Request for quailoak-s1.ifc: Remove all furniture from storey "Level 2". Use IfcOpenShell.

First a look at what the model holds.

```python
import ifcopenshell
import ifcopenshell.util.element

model = ifcopenshell.open("quailoak-s1.ifc")
print(model.schema)
storey = next(s for s in model.by_type("IfcBuildingStorey") if s.Name == "Level 2")
furniture = [e for e in ifcopenshell.util.element.get_decomposition(storey) if e.is_a("IfcFurnishingElement")]
seen = {}
for e in furniture:
    element_type = ifcopenshell.util.element.get_type(e)
    name = element_type.Name if element_type not in (None, e) else None
    seen[name] = seen.get(name, 0) + 1
for name, count in sorted(seen.items(), key=str):
    print(count, "x", name)
```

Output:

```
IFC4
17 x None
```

```python
import ifcopenshell
import ifcopenshell.api.root
import ifcopenshell.util.element

model = ifcopenshell.open("quailoak-s1.ifc")

storey = next(s for s in model.by_type("IfcBuildingStorey") if s.Name == "Level 2")
furniture = [e for e in ifcopenshell.util.element.get_decomposition(storey) if e.is_a("IfcFurnishingElement")]

for e in furniture:
    ifcopenshell.api.root.remove_product(model, product=e)
print(len(furniture), "removed")

model.write("quailoak-s1_rev.ifc")
```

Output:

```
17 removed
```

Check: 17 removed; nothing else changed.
